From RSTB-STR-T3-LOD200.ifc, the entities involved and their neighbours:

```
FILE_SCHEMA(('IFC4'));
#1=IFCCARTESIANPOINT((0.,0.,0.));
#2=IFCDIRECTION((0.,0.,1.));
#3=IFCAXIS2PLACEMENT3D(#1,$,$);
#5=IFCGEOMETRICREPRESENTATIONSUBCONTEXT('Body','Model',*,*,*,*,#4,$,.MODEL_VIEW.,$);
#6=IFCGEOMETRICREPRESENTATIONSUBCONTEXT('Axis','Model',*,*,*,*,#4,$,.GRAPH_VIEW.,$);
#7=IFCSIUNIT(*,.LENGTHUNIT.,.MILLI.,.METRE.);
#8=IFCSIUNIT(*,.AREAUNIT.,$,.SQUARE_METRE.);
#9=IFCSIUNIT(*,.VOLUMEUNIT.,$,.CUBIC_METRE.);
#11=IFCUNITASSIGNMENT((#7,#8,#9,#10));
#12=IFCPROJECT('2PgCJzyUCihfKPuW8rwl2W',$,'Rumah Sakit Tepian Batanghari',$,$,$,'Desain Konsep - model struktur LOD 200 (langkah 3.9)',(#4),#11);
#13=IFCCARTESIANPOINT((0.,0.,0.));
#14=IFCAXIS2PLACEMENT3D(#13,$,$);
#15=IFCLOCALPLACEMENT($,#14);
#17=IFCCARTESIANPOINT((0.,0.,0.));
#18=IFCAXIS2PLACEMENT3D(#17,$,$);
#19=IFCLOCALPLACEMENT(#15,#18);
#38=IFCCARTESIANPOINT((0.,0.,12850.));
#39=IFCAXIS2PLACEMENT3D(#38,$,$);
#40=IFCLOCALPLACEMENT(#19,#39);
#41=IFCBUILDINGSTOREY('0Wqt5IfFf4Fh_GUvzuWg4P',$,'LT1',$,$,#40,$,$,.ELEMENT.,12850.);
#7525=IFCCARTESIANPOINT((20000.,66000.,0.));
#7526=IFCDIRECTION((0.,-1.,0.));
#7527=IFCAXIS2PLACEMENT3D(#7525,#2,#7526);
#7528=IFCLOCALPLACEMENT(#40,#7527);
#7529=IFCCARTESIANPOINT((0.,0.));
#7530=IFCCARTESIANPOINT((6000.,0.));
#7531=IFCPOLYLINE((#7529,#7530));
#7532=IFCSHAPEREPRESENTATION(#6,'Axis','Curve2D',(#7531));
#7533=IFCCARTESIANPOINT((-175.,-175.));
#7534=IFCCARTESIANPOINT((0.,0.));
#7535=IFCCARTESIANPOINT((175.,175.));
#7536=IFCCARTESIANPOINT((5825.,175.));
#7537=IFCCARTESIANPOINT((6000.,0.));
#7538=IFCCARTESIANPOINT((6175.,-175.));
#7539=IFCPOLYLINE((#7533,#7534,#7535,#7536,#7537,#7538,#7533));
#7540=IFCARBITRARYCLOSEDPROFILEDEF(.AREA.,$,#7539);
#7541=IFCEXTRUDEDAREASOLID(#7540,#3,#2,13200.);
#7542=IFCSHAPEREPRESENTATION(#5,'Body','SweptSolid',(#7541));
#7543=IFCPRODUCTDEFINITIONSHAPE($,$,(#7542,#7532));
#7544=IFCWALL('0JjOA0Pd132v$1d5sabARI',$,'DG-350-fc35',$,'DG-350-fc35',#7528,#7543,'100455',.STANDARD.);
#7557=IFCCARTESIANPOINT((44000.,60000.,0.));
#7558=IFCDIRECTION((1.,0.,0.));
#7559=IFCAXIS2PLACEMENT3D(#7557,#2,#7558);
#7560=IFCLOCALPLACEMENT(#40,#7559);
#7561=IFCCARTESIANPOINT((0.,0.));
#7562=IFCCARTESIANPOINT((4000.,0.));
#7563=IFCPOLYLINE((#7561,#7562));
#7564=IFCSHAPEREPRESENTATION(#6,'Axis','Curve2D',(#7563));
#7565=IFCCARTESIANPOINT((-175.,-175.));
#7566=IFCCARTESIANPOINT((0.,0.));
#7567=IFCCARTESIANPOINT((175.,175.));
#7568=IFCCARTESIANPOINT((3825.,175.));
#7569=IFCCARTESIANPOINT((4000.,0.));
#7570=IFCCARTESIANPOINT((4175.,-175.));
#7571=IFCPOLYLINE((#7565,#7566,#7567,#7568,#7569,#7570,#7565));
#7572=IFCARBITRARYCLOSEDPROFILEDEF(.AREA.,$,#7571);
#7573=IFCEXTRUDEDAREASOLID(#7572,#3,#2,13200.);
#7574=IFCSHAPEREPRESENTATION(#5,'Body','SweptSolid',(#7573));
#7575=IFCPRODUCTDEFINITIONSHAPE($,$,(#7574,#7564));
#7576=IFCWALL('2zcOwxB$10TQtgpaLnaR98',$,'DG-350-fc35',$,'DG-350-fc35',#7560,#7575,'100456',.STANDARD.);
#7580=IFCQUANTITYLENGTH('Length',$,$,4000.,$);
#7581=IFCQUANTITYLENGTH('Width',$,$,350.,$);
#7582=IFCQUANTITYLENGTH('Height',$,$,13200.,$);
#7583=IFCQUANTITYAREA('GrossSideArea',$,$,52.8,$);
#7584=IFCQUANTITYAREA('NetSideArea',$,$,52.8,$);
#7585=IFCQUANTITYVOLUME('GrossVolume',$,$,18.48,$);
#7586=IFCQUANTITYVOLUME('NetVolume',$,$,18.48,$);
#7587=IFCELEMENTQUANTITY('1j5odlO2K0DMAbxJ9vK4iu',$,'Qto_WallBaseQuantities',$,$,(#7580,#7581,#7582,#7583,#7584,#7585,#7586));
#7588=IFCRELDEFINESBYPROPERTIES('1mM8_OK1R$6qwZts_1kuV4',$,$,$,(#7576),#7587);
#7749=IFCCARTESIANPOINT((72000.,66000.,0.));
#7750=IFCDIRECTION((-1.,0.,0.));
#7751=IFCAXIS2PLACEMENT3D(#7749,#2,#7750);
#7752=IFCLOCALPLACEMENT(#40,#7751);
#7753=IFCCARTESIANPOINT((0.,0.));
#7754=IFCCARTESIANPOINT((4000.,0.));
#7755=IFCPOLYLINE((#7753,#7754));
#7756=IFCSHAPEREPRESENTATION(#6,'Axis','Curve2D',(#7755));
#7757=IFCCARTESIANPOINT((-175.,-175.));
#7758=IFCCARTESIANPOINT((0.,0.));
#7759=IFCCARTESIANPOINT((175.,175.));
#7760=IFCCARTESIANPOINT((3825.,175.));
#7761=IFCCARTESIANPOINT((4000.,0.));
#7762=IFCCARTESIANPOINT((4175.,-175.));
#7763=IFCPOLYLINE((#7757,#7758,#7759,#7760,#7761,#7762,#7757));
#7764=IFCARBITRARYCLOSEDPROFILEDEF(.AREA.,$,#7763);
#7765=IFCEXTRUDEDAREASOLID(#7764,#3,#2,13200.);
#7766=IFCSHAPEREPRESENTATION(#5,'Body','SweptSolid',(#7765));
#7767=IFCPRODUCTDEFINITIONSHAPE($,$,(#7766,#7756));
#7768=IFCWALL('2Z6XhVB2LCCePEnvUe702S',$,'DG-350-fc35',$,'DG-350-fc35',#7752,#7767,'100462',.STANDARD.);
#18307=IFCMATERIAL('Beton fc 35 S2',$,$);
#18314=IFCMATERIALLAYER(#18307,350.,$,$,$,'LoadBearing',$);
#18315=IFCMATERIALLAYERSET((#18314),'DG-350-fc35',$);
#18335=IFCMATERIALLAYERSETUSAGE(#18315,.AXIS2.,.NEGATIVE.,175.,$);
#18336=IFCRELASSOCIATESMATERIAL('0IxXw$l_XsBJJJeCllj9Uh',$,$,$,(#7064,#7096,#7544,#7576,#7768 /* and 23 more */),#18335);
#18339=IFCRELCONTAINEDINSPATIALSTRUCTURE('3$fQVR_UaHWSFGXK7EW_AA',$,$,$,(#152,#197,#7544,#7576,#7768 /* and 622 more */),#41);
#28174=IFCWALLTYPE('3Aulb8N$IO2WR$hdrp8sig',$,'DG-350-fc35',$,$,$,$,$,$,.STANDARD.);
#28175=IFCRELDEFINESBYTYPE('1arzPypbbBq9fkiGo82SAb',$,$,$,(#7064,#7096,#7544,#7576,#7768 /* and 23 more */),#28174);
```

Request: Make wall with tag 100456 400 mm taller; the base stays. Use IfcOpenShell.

```python
import ifcopenshell
import ifcopenshell.api.pset
import ifcopenshell.geom
import ifcopenshell.util.element
import ifcopenshell.util.representation
import ifcopenshell.util.shape
import ifcopenshell.util.unit

model = ifcopenshell.open("RSTB-STR-T3-LOD200.ifc")
unit_scale = ifcopenshell.util.unit.calculate_unit_scale(model)
area_scale = ifcopenshell.util.unit.calculate_unit_scale(model, "AREAUNIT")
volume_scale = ifcopenshell.util.unit.calculate_unit_scale(model, "VOLUMEUNIT")
settings = ifcopenshell.geom.settings()


def volume(element):
    """Net volume in cubic metres, openings subtracted."""
    shape = ifcopenshell.geom.create_shape(settings, element)
    return ifcopenshell.util.shape.get_volume(shape.geometry)


wall = model.by_guid("2zcOwxB$10TQtgpaLnaR98")
before = volume(wall)

body = ifcopenshell.util.representation.get_representation(wall, "Model", "Body")
solid = body.Items[0]
old_height = solid.Depth
solid.Depth += 0.4 / unit_scale
after = volume(wall)
thickness = 0.35  # wall thickness in metres

# Update the stored height, areas and volumes.
qto = model.by_id(ifcopenshell.util.element.get_pset(wall, "Qto_WallBaseQuantities", should_inherit=False)["id"])
ifcopenshell.api.pset.edit_qto(model, qto=qto, properties={
    "Height": solid.Depth,
    "GrossSideArea": ifcopenshell.util.element.get_pset(wall, "Qto_WallBaseQuantities", "GrossSideArea") * solid.Depth / old_height,
    "NetSideArea": after / thickness / area_scale,
    "GrossVolume": ifcopenshell.util.element.get_pset(wall, "Qto_WallBaseQuantities", "GrossVolume") * solid.Depth / old_height,
    "NetVolume": after / volume_scale,
})

print(f"height {old_height:g} -> {solid.Depth:g}, volume {before:.3f} -> {after:.3f} m3")

model.write("RSTB-STR-T3-LOD200_edited.ifc")
```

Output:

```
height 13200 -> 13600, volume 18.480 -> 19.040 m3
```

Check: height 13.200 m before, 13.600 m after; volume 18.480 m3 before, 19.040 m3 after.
